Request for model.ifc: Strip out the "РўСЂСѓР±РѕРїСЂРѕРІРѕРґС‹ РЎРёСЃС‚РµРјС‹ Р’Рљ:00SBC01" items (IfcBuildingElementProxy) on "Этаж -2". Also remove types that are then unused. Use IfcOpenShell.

First a look at what the model holds.

```python
import ifcopenshell
import ifcopenshell.util.element

model = ifcopenshell.open("model.ifc")
print(model.schema)
storey = next(s for s in model.by_type("IfcBuildingStorey") if s.Name == "Этаж -2")
proxies = [e for e in ifcopenshell.util.element.get_decomposition(storey) if e.is_a("IfcBuildingElementProxy")]
seen = {}
for e in proxies:
    element_type = ifcopenshell.util.element.get_type(e)
    name = element_type.Name if element_type not in (None, e) else None
    seen[name] = seen.get(name, 0) + 1
for name, count in sorted(seen.items(), key=str):
    print(count, "x", name)
```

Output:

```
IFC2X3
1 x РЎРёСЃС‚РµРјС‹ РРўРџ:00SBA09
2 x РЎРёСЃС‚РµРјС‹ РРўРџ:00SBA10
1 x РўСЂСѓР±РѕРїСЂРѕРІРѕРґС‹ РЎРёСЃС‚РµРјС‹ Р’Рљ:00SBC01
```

```python
import ifcopenshell
import ifcopenshell.api.root
import ifcopenshell.util.element

model = ifcopenshell.open("model.ifc")

storey = next(s for s in model.by_type("IfcBuildingStorey") if s.Name == "Этаж -2")
proxies = [e for e in ifcopenshell.util.element.get_decomposition(storey) if e.is_a("IfcBuildingElementProxy")]
targets = [e for e in proxies if (t := ifcopenshell.util.element.get_type(e)) not in (None, e) and t.Name == "РўСЂСѓР±РѕРїСЂРѕРІРѕРґС‹ РЎРёСЃС‚РµРјС‹ Р’Рљ:00SBC01"]
types = {ifcopenshell.util.element.get_type(e) for e in targets} - {None, *targets}

for e in targets:
    ifcopenshell.api.root.remove_product(model, product=e)
print(len(targets), "removed")

unused = [t for t in types if not ifcopenshell.util.element.get_types(t)]
for t in unused:
    ifcopenshell.api.root.remove_product(model, product=t)
print(len(unused), "unused types removed")

model.write("model_v2.ifc")
```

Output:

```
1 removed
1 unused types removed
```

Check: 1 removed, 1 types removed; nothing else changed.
